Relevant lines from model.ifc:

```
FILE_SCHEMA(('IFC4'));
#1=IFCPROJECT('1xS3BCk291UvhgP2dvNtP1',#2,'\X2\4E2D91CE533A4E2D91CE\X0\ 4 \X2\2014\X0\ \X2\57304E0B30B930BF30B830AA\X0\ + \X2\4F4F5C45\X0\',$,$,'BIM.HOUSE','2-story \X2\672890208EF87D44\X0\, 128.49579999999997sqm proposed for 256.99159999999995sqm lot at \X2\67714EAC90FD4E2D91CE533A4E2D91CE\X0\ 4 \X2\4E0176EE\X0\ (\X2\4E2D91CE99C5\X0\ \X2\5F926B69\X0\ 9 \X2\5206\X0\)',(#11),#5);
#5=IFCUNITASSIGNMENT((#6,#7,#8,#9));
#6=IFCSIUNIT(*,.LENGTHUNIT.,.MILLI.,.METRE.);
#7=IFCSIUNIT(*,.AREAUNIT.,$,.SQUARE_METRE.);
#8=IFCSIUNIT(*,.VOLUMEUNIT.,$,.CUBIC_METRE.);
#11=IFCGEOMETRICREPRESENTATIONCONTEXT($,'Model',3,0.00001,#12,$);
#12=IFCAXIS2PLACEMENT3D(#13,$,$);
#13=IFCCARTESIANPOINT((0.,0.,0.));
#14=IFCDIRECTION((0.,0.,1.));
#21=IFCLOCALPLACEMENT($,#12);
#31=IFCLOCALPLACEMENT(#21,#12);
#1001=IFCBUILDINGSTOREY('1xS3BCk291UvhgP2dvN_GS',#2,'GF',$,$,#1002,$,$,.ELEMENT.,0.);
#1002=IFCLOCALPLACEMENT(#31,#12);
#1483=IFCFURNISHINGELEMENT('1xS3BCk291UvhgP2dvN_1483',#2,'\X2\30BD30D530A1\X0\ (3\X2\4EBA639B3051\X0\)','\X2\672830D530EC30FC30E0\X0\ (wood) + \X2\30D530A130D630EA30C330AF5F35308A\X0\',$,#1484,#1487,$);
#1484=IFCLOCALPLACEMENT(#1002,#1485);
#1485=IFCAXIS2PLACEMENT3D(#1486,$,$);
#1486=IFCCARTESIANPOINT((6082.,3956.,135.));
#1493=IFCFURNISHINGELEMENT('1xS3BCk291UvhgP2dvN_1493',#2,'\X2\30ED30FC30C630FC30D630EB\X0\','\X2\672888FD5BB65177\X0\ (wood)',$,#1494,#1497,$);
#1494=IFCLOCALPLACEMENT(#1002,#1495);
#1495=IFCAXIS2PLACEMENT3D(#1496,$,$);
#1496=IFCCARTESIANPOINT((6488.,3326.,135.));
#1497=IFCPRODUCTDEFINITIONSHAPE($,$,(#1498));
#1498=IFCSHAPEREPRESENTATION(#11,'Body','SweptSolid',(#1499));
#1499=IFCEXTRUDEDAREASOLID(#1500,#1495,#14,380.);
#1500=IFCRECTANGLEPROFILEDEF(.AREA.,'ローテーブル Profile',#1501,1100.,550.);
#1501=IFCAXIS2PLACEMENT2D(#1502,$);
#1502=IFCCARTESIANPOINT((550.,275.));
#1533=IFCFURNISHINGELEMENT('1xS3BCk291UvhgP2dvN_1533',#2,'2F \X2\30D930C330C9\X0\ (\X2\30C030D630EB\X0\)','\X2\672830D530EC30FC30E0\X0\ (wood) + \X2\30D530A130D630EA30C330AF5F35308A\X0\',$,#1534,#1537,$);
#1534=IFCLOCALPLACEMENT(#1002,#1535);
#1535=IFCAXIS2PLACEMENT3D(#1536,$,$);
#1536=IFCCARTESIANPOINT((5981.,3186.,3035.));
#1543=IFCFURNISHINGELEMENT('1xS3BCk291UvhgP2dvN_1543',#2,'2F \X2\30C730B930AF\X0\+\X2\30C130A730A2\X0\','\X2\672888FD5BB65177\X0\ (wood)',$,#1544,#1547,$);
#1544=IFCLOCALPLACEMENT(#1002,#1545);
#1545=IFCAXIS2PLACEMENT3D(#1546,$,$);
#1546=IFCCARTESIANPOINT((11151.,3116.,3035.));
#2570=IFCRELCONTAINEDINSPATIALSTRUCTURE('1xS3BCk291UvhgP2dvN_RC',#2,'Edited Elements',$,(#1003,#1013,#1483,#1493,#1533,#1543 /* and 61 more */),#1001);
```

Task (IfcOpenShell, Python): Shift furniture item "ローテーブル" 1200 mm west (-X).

```python
import ifcopenshell
import ifcopenshell.api.geometry
import ifcopenshell.util.placement

model = ifcopenshell.open("model.ifc")

item = model.by_id(1493)
matrix = ifcopenshell.util.placement.get_local_placement(item.ObjectPlacement)
matrix[0, 3] -= 1200.0
ifcopenshell.api.geometry.edit_object_placement(model, product=item, matrix=matrix, is_si=False)

print(ifcopenshell.util.placement.get_local_placement(item.ObjectPlacement).round(3) + 0.0)

model.write("model_updated.ifc")
```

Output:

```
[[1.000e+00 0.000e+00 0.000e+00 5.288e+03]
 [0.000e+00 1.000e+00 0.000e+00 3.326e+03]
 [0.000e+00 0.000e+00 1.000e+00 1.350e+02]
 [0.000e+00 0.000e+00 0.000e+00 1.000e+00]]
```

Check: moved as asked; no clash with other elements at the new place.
